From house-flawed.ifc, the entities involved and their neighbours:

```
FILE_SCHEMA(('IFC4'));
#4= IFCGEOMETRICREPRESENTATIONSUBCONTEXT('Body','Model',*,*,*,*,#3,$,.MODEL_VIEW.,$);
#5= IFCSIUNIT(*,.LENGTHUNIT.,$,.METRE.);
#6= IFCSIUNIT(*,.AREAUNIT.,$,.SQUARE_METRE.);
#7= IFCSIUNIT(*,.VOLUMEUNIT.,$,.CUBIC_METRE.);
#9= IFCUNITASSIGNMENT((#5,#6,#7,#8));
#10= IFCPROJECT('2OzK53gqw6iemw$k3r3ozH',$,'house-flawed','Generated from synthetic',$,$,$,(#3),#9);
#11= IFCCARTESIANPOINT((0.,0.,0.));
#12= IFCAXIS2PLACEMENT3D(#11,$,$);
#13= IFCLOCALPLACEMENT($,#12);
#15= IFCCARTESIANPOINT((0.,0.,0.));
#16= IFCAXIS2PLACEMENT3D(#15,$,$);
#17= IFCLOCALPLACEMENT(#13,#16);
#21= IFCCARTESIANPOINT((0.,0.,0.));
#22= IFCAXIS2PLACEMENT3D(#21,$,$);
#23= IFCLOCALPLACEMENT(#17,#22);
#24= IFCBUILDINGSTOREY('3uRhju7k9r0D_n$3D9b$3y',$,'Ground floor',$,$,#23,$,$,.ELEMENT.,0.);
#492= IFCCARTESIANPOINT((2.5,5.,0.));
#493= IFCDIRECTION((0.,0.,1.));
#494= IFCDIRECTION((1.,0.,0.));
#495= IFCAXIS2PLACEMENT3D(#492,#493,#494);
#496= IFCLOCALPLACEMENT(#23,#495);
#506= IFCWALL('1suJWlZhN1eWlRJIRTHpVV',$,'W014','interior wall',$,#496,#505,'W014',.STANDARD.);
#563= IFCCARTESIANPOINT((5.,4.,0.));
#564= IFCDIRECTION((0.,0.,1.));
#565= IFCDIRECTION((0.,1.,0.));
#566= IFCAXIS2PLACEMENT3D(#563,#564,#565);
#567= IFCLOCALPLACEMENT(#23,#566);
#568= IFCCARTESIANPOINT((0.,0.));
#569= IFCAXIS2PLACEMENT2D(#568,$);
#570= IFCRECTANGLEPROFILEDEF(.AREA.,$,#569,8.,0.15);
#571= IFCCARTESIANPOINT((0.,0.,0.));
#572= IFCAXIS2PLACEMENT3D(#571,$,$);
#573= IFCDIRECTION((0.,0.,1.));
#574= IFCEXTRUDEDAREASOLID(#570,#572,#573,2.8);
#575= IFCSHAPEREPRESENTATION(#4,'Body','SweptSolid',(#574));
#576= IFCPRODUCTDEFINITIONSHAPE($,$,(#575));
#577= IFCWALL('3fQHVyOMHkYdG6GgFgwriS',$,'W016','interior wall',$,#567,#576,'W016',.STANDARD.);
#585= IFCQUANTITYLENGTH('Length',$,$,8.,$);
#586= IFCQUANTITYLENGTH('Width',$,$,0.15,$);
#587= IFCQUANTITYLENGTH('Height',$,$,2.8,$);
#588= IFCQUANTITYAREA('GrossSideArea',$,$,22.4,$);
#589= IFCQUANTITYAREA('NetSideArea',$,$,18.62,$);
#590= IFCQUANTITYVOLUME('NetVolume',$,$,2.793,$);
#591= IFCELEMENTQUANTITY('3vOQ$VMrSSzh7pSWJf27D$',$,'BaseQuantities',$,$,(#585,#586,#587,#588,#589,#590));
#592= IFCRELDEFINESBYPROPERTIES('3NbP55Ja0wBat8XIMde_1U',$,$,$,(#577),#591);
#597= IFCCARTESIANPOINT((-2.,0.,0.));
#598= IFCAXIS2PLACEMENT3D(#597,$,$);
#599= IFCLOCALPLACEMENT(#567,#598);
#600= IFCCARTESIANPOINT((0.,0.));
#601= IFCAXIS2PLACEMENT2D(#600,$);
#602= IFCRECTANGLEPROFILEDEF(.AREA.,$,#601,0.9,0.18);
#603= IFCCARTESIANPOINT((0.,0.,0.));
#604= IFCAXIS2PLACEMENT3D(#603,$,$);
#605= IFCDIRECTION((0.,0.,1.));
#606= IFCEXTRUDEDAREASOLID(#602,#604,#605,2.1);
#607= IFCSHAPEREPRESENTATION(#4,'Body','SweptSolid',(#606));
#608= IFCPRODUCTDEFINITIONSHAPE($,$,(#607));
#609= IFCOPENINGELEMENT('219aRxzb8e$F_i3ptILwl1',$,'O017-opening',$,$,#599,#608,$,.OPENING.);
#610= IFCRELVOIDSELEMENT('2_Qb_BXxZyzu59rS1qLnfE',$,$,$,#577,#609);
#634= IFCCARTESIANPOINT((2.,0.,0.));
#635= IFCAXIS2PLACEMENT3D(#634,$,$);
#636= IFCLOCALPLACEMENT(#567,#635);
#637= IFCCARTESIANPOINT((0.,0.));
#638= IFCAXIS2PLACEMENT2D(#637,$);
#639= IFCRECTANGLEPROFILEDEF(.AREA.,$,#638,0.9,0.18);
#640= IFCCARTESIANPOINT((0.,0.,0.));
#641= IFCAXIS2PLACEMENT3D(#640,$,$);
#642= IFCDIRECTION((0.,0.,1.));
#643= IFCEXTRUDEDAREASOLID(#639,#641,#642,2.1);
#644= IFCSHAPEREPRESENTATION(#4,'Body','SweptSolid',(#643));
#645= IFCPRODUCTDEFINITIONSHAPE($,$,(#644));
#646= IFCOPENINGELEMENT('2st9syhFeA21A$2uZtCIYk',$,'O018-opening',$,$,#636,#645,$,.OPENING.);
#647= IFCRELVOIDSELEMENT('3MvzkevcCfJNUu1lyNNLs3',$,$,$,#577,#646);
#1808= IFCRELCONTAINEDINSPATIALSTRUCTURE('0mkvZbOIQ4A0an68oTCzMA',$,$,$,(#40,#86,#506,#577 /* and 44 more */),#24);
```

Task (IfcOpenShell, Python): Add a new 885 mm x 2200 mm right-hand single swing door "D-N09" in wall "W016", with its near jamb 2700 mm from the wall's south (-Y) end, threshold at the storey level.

```python
import numpy as np
import ifcopenshell
import ifcopenshell.api.feature
import ifcopenshell.api.geometry
import ifcopenshell.api.pset
import ifcopenshell.api.root
import ifcopenshell.api.spatial
import ifcopenshell.geom
import ifcopenshell.util.element
import ifcopenshell.util.placement
import ifcopenshell.util.representation
import ifcopenshell.util.shape
import ifcopenshell.util.unit

model = ifcopenshell.open("house-flawed.ifc")
unit_scale = ifcopenshell.util.unit.calculate_unit_scale(model)
area_scale = ifcopenshell.util.unit.calculate_unit_scale(model, "AREAUNIT")
volume_scale = ifcopenshell.util.unit.calculate_unit_scale(model, "VOLUMEUNIT")
settings = ifcopenshell.geom.settings()


def volume(element):
    """Net volume in cubic metres, openings subtracted."""
    shape = ifcopenshell.geom.create_shape(settings, element)
    return ifcopenshell.util.shape.get_volume(shape.geometry)


wall = model.by_guid("3fQHVyOMHkYdG6GgFgwriS")
storey = ifcopenshell.util.element.get_container(wall, ifc_class="IfcBuildingStorey")
context = ifcopenshell.util.representation.get_context(model, "Model", "Body", "MODEL_VIEW")
before = volume(wall)

width, height, from_end, sill = 0.885, 2.2, 2.7, 0.0  # metres

# The wall runs along its own X axis, and the end named is its -X end.
wall_shape = ifcopenshell.geom.create_shape(settings, wall)
x, y, z = ifcopenshell.util.shape.get_vertices(wall_shape.geometry).T
start = x.min() + from_end
face, thickness = float(y.min()), float(y.max() - y.min())
wall_matrix = ifcopenshell.util.placement.get_local_placement(wall.ObjectPlacement)
level = ifcopenshell.util.placement.get_local_placement(storey.ObjectPlacement)[2, 3]


def in_wall(x, y):
    """Placement at x, y metres in the wall's axes, at sill height."""
    matrix = wall_matrix.copy()
    matrix[:, 3] = wall_matrix @ np.array([x / unit_scale, y / unit_scale, 0.0, 1.0])
    matrix[2, 3] = level + sill / unit_scale
    return matrix


# Opening: a box that overshoots both wall faces by 50 mm.
opening = ifcopenshell.api.root.create_entity(model, ifc_class="IfcOpeningElement", predefined_type="OPENING")
box = ifcopenshell.api.geometry.add_wall_representation(
    model, context=context, length=width, height=height, thickness=thickness + 0.1
)
ifcopenshell.api.geometry.assign_representation(model, product=opening, representation=box)
ifcopenshell.api.geometry.edit_object_placement(model, product=opening, matrix=in_wall(start, face - 0.05), is_si=False)
ifcopenshell.api.feature.add_feature(model, feature=opening, element=wall)

door = ifcopenshell.api.root.create_entity(model, ifc_class="IfcDoor", name="D-N09", predefined_type="DOOR")
door.OverallWidth, door.OverallHeight = width / unit_scale, height / unit_scale
door.OperationType = "SINGLE_SWING_RIGHT"
body = ifcopenshell.api.geometry.add_door_representation(
    model,
    context=context,
    overall_width=door.OverallWidth,
    overall_height=door.OverallHeight,
    operation_type="SINGLE_SWING_RIGHT",
    lining_properties={"LiningDepth": thickness / unit_scale, "ThresholdDepth": thickness / unit_scale},
)
ifcopenshell.api.geometry.assign_representation(model, product=door, representation=body)
ifcopenshell.api.spatial.assign_container(model, products=[door], relating_structure=storey)
ifcopenshell.api.feature.add_filling(model, opening=opening, element=door)

# The lining spans the wall, so the door starts at the wall face.
ifcopenshell.api.geometry.edit_object_placement(model, product=door, matrix=in_wall(start, face), is_si=False)

after = volume(wall)

# Update the wall's stored quantities.
qto = model.by_id(ifcopenshell.util.element.get_pset(wall, "BaseQuantities", should_inherit=False)["id"])
ifcopenshell.api.pset.edit_qto(model, qto=qto, properties={
    "NetSideArea": after / thickness / area_scale,
    "NetVolume": after / volume_scale,
})

print(f"wall volume {before:.3f} -> {after:.3f} m3")

model.write("house-flawed_v2.ifc")
```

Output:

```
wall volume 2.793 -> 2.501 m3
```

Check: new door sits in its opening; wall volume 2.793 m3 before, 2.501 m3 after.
